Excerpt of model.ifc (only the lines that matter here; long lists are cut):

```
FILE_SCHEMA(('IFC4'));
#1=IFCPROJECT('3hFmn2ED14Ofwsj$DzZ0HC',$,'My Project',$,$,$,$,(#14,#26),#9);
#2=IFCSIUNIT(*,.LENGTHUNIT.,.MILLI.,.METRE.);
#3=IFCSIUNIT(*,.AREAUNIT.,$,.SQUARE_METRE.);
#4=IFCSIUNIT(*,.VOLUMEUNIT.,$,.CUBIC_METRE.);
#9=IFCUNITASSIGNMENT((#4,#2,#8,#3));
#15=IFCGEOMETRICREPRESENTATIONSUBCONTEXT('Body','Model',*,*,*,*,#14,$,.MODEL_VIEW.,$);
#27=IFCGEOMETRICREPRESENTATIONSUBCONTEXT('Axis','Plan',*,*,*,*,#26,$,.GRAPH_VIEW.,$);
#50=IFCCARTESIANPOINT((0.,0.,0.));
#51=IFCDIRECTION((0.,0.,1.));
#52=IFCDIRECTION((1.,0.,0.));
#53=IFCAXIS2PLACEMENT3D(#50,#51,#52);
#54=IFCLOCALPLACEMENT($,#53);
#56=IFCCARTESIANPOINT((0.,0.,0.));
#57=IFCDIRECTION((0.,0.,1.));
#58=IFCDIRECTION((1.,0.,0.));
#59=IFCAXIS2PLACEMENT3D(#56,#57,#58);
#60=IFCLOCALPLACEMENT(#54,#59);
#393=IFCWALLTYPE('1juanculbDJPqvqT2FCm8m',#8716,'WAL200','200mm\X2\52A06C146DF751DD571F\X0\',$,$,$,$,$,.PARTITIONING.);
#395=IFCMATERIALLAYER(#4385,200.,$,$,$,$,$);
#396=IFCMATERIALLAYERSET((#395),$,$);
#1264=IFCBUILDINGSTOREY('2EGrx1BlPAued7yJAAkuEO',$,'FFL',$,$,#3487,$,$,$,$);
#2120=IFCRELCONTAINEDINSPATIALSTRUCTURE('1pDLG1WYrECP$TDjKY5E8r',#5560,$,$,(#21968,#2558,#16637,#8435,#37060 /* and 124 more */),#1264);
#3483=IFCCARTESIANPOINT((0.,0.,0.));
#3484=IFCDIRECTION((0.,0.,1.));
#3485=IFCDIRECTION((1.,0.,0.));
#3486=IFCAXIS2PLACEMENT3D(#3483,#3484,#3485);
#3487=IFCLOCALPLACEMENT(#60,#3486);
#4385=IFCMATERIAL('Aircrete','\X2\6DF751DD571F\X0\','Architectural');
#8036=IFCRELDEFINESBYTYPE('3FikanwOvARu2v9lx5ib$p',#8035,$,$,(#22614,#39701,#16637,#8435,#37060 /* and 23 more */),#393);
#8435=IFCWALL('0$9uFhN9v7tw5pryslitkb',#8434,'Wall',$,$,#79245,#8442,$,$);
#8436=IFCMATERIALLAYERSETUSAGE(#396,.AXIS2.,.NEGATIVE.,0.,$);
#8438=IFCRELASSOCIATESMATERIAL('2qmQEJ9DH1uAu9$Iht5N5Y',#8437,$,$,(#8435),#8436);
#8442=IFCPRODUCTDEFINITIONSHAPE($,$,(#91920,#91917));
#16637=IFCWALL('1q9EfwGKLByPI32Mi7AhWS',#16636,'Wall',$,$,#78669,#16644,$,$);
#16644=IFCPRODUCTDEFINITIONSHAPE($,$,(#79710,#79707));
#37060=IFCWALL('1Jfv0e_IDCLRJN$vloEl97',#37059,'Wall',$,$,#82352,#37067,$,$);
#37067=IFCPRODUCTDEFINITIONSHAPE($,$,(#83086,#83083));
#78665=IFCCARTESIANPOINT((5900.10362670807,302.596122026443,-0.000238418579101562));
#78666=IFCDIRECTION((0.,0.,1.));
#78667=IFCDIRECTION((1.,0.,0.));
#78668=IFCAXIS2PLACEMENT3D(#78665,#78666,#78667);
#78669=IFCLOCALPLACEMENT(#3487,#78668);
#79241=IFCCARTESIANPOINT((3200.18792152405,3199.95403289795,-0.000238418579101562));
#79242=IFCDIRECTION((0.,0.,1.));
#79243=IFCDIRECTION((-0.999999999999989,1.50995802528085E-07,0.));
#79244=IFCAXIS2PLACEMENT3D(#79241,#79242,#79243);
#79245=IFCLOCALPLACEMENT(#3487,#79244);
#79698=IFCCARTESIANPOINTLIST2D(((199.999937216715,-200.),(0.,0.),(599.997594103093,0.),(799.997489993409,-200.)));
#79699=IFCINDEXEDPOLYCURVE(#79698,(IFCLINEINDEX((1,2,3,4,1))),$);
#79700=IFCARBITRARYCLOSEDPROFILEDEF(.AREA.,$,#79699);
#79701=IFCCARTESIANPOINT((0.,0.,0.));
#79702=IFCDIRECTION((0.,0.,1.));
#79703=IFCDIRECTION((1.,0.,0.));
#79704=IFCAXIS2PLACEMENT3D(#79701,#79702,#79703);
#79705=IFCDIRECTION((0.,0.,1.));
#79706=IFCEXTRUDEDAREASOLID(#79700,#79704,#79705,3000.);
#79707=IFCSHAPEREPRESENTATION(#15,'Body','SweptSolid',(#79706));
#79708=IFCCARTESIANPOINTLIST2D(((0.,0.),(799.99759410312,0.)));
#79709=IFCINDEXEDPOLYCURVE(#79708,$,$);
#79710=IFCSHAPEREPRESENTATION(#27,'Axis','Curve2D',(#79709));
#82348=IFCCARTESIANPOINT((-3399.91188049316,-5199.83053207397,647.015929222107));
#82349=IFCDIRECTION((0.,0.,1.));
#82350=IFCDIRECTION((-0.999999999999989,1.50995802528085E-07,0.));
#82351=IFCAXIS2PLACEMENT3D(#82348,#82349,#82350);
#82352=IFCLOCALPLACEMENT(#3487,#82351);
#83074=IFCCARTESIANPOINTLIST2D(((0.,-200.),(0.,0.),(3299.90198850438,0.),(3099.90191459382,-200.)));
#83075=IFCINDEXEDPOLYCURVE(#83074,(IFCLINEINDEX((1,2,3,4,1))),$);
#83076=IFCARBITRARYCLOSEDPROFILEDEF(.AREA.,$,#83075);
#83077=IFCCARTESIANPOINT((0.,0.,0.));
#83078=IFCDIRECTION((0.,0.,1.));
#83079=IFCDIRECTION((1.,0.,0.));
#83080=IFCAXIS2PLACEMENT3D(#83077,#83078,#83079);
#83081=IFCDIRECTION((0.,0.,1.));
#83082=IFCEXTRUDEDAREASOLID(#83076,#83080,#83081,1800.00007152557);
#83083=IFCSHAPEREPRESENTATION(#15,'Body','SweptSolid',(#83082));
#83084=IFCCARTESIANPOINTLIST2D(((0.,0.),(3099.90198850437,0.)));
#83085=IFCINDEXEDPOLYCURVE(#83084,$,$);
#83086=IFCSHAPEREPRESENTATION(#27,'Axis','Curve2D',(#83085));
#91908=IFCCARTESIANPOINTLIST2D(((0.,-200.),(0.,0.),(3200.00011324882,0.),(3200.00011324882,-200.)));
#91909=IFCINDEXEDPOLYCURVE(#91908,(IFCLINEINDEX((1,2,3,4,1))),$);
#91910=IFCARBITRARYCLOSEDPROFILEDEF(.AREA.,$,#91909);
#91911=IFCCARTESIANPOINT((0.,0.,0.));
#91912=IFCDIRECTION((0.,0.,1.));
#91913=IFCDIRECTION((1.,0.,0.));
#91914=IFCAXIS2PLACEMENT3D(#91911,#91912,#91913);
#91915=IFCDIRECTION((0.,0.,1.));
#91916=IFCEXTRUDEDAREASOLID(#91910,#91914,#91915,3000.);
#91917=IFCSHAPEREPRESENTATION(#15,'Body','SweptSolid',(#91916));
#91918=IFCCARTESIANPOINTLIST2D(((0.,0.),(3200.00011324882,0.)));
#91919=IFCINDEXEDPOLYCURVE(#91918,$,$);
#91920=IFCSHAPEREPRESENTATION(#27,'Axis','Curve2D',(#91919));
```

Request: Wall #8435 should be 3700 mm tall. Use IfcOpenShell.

```python
import ifcopenshell
import ifcopenshell.geom
import ifcopenshell.util.representation
import ifcopenshell.util.shape
import ifcopenshell.util.unit

model = ifcopenshell.open("model.ifc")
unit_scale = ifcopenshell.util.unit.calculate_unit_scale(model)
settings = ifcopenshell.geom.settings()


def volume(element):
    """Net volume in cubic metres, openings subtracted."""
    shape = ifcopenshell.geom.create_shape(settings, element)
    return ifcopenshell.util.shape.get_volume(shape.geometry)


wall = model.by_guid("0$9uFhN9v7tw5pryslitkb")
before = volume(wall)

body = ifcopenshell.util.representation.get_representation(wall, "Model", "Body")
solid = body.Items[0]
old_height = solid.Depth
solid.Depth = 3.7 / unit_scale
after = volume(wall)

print(f"height {old_height:g} -> {solid.Depth:g}, volume {before:.3f} -> {after:.3f} m3")

model.write("model_v2.ifc")
```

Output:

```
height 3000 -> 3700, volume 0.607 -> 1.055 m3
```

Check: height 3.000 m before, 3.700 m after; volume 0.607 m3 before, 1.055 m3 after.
